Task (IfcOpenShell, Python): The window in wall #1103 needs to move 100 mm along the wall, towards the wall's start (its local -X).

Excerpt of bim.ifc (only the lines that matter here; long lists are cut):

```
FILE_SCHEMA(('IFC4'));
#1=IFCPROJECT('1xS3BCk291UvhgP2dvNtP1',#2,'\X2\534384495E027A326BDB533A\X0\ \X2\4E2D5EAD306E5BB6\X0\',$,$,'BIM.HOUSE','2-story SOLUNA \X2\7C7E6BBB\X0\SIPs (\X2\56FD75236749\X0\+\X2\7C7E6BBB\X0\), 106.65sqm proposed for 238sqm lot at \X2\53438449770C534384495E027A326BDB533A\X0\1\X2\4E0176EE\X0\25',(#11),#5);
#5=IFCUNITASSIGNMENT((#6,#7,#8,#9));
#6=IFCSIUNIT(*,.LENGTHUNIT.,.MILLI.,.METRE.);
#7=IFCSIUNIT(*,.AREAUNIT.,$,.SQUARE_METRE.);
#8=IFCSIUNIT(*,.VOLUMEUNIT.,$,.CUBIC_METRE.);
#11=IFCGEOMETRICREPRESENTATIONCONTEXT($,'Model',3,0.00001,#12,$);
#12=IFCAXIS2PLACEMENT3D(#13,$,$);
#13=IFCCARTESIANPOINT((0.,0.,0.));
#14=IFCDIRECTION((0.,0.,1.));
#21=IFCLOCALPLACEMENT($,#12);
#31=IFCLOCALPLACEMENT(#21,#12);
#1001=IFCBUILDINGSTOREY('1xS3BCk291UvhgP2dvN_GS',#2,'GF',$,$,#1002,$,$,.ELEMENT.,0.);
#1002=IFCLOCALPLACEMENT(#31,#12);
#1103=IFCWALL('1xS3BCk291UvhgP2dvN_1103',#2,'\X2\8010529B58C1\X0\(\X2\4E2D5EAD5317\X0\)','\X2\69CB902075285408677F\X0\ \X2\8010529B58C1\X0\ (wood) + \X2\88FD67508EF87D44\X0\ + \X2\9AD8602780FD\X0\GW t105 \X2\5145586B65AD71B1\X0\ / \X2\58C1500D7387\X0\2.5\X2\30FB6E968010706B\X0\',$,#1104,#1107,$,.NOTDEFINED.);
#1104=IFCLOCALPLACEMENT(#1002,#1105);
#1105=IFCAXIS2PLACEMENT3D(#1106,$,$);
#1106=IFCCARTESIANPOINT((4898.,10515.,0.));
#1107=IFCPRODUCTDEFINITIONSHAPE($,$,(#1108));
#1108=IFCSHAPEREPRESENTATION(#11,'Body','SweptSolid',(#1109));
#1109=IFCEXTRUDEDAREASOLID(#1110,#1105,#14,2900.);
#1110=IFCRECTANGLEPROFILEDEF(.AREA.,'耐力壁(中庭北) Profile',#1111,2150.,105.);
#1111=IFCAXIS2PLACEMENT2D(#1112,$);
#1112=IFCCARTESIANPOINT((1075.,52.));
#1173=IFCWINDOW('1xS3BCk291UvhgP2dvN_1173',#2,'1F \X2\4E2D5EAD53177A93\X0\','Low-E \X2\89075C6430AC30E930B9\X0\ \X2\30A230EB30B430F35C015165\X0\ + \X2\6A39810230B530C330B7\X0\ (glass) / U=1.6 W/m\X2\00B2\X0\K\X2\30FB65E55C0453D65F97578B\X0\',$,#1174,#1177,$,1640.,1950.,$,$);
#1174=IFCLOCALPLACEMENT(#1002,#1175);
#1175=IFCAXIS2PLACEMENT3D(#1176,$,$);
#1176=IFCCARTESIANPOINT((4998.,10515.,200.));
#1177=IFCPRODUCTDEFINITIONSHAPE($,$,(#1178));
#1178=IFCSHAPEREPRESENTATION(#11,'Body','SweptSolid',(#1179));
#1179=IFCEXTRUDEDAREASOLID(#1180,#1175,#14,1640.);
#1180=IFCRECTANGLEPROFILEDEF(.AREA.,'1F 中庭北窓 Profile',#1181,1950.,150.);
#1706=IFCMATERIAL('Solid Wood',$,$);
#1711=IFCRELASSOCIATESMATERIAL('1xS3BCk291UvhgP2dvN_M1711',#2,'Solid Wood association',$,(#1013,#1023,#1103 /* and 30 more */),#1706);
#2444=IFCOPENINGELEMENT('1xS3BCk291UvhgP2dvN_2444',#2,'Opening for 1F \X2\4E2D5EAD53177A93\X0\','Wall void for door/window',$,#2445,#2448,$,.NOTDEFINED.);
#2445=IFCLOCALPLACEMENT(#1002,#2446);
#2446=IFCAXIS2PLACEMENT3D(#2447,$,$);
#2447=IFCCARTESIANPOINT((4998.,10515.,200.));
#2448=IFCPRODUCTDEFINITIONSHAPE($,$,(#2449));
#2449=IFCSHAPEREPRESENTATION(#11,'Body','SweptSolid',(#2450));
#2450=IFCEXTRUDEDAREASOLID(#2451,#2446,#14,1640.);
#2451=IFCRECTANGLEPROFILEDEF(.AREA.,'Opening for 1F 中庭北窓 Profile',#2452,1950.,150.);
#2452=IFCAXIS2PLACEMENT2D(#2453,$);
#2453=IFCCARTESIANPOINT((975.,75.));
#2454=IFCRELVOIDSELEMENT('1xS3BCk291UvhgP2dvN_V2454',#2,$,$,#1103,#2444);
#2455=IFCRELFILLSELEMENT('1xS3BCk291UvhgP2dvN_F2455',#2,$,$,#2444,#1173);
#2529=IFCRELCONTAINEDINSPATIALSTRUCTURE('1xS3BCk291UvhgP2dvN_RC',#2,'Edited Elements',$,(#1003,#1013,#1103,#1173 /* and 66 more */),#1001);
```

```python
import ifcopenshell
import ifcopenshell.api.geometry
import ifcopenshell.util.placement

model = ifcopenshell.open("bim.ifc")

window = model.by_guid("1xS3BCk291UvhgP2dvN_1173")
opening = window.FillsVoids[0].RelatingOpeningElement
wall = opening.VoidsElements[0].RelatingBuildingElement

wall_matrix = ifcopenshell.util.placement.get_local_placement(wall.ObjectPlacement)
shift = wall_matrix[:3, 0] * -100.0
before = ifcopenshell.util.placement.get_local_placement(window.ObjectPlacement)[:3, 3].copy()

# The window is not placed relative to its opening, so move both.
for product in (opening, window):
    matrix = ifcopenshell.util.placement.get_local_placement(product.ObjectPlacement)
    matrix[:3, 3] += shift
    ifcopenshell.api.geometry.edit_object_placement(model, product=product, matrix=matrix, is_si=False)

after = ifcopenshell.util.placement.get_local_placement(window.ObjectPlacement)[:3, 3]
print("window moved by", (after - before).round(3) + 0.0)

model.write("bim-out.ifc")
```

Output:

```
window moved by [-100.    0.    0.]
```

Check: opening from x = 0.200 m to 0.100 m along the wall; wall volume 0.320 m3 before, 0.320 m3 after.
